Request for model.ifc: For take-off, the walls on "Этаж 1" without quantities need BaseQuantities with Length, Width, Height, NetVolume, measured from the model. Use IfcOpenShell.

First a look at what the model holds.

```python
import ifcopenshell
import ifcopenshell.util.element
import ifcopenshell.util.unit

model = ifcopenshell.open("model.ifc")
print(model.schema)
for unit_type in ("LENGTHUNIT", "AREAUNIT", "VOLUMEUNIT"):
    print(unit_type, ifcopenshell.util.unit.calculate_unit_scale(model, unit_type))
storey = next(s for s in model.by_type("IfcBuildingStorey") if s.Name == "Этаж 1")
walls = [e for e in ifcopenshell.util.element.get_decomposition(storey) if e.is_a("IfcWall")]
for e in sorted(walls, key=lambda e: e.id()):
    print(e.id(), e.is_a(), e.Name, list(ifcopenshell.util.element.get_psets(e, qtos_only=True)), sep=" | ")
```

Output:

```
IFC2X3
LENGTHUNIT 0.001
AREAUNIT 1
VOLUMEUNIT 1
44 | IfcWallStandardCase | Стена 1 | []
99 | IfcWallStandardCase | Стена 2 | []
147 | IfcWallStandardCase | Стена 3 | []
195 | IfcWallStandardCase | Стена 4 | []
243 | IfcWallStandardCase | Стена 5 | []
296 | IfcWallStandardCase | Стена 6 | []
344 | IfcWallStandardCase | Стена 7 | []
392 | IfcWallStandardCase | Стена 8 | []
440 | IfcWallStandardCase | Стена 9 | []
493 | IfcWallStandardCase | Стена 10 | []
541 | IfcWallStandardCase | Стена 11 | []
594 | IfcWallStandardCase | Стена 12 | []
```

```python
import ifcopenshell
import ifcopenshell.api.pset
import ifcopenshell.geom
import ifcopenshell.util.element
import ifcopenshell.util.shape
import ifcopenshell.util.unit

model = ifcopenshell.open("model.ifc")
unit_scale = ifcopenshell.util.unit.calculate_unit_scale(model)
volume_scale = ifcopenshell.util.unit.calculate_unit_scale(model, "VOLUMEUNIT")
settings = ifcopenshell.geom.settings()

storey = next(s for s in model.by_type("IfcBuildingStorey") if s.Name == "Этаж 1")
walls = [e for e in ifcopenshell.util.element.get_decomposition(storey) if e.is_a("IfcWall")]

for e in sorted(walls, key=lambda e: e.id()):
    if ifcopenshell.util.element.get_psets(e, qtos_only=True, should_inherit=False):
        continue
    # Geometry comes back in metres, in the element's own axes.
    shape = ifcopenshell.geom.create_shape(settings, e)
    values = {
        "Length": ifcopenshell.util.shape.get_x(shape.geometry) / unit_scale,
        "Width": ifcopenshell.util.shape.get_y(shape.geometry) / unit_scale,
        "Height": ifcopenshell.util.shape.get_z(shape.geometry) / unit_scale,
        "NetVolume": ifcopenshell.util.shape.get_volume(shape.geometry) / volume_scale,
    }
    qto = ifcopenshell.api.pset.add_qto(model, product=e, name="BaseQuantities")
    ifcopenshell.api.pset.edit_qto(model, qto=qto, properties=values)
    print(e.id(), {k: round(v, 3) for k, v in values.items()})

model.write("model_edited.ifc")
```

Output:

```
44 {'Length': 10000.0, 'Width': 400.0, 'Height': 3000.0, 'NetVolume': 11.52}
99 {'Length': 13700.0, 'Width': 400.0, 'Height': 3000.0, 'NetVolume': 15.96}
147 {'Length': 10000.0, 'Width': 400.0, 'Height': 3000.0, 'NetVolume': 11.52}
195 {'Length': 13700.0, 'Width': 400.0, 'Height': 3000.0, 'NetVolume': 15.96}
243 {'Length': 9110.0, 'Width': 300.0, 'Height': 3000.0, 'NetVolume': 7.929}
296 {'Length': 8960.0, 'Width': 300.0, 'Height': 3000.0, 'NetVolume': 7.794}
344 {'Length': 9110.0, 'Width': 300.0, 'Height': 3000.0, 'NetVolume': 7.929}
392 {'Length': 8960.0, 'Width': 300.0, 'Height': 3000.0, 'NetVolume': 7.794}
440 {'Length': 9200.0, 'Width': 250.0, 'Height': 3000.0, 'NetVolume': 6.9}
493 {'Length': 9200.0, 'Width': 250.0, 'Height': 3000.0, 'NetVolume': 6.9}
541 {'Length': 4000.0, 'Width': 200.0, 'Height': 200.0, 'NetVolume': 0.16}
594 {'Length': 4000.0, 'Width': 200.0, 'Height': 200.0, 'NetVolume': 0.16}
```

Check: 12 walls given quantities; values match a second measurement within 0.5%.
